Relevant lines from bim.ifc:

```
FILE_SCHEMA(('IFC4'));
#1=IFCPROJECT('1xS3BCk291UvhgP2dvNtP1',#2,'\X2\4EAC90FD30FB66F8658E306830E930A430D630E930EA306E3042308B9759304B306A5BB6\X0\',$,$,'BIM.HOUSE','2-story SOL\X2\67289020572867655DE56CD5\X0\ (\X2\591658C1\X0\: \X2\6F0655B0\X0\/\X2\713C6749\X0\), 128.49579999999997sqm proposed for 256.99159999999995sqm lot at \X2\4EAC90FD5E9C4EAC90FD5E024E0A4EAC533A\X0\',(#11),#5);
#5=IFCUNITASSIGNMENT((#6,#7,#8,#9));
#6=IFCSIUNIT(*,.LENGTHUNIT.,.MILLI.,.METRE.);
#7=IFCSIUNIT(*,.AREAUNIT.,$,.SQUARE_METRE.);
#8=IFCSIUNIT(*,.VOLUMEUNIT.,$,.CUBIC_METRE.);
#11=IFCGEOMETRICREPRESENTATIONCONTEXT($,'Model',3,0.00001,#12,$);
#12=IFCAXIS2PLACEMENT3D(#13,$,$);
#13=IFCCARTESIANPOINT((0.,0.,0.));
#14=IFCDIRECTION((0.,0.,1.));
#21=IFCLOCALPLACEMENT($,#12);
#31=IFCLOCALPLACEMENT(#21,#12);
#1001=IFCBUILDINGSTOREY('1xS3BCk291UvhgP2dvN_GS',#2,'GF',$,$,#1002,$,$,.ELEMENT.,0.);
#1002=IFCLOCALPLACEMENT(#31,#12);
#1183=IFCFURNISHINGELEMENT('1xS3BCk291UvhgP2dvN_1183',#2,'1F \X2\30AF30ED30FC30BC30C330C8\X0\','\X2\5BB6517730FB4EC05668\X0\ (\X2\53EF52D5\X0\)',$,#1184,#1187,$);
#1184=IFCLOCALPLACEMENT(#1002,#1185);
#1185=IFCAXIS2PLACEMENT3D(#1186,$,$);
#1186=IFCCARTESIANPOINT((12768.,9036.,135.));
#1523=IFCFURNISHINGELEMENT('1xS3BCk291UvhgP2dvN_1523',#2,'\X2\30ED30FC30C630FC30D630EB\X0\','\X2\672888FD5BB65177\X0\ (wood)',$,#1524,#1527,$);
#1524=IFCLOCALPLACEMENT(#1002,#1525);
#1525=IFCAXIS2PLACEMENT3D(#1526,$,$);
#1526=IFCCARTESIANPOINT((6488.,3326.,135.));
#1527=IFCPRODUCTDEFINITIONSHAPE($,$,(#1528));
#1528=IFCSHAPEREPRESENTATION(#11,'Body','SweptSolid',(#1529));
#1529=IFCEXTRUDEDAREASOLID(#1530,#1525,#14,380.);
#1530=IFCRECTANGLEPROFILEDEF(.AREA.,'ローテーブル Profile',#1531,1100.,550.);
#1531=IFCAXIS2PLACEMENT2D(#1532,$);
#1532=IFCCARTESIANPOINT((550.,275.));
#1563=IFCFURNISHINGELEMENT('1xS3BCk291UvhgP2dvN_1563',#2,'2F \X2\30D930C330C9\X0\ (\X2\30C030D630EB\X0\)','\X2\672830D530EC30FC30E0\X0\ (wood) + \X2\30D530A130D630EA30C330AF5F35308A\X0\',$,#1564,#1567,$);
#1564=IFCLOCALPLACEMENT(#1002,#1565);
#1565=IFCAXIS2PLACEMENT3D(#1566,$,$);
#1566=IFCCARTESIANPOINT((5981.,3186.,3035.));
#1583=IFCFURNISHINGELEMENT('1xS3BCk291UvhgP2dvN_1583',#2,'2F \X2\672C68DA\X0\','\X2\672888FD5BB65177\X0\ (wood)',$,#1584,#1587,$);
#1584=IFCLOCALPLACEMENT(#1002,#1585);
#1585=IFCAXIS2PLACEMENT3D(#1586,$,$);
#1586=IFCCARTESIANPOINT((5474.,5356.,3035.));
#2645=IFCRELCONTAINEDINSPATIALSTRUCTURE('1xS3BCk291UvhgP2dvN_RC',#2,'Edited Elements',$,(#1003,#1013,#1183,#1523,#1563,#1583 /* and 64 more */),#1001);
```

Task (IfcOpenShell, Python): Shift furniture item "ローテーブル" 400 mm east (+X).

```python
import ifcopenshell
import ifcopenshell.api.geometry
import ifcopenshell.util.placement
import ifcopenshell.util.unit

model = ifcopenshell.open("bim.ifc")
unit_scale = ifcopenshell.util.unit.calculate_unit_scale(model)

item = model.by_guid("1xS3BCk291UvhgP2dvN_1523")
matrix = ifcopenshell.util.placement.get_local_placement(item.ObjectPlacement)
matrix[0, 3] += 0.4 / unit_scale
ifcopenshell.api.geometry.edit_object_placement(model, product=item, matrix=matrix, is_si=False)

print(ifcopenshell.util.placement.get_local_placement(item.ObjectPlacement).round(3) + 0.0)

model.write("bim_updated.ifc")
```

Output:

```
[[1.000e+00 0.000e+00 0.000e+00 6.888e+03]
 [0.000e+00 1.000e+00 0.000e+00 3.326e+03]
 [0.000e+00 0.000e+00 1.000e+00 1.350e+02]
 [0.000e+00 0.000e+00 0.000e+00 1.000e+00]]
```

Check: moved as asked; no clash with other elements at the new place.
